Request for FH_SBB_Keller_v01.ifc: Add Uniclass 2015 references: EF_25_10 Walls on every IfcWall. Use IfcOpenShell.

First a look at what the model holds.

```python
import ifcopenshell

model = ifcopenshell.open("FH_SBB_Keller_v01.ifc")
print(model.schema)
print("classifications:", [c.Name for c in model.by_type("IfcClassification")])
for ifc_class in ("IfcDoor", "IfcRoof", "IfcStair", "IfcWall", "IfcWindow"):
    print(ifc_class, len(model.by_type(ifc_class)))
```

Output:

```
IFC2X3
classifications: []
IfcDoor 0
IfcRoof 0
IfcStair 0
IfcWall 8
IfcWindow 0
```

```python
import ifcopenshell
import ifcopenshell.api.classification

model = ifcopenshell.open("FH_SBB_Keller_v01.ifc")

# IFC2X3 requires Source and Edition and has no link from the project to the system.
system = model.create_entity("IfcClassification", Source="NBS", Edition="2015", Name="Uniclass 2015")

codes = {
    "IfcWall": ("EF_25_10", "Walls"),
}
for ifc_class, (code, name) in codes.items():
    products = model.by_type(ifc_class)
    ifcopenshell.api.classification.add_reference(
        model, products=products, classification=system, identification=code, name=name
    )
    print(code, len(products))

model.write("FH_SBB_Keller_v01-out.ifc")
```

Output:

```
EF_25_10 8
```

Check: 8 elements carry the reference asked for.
